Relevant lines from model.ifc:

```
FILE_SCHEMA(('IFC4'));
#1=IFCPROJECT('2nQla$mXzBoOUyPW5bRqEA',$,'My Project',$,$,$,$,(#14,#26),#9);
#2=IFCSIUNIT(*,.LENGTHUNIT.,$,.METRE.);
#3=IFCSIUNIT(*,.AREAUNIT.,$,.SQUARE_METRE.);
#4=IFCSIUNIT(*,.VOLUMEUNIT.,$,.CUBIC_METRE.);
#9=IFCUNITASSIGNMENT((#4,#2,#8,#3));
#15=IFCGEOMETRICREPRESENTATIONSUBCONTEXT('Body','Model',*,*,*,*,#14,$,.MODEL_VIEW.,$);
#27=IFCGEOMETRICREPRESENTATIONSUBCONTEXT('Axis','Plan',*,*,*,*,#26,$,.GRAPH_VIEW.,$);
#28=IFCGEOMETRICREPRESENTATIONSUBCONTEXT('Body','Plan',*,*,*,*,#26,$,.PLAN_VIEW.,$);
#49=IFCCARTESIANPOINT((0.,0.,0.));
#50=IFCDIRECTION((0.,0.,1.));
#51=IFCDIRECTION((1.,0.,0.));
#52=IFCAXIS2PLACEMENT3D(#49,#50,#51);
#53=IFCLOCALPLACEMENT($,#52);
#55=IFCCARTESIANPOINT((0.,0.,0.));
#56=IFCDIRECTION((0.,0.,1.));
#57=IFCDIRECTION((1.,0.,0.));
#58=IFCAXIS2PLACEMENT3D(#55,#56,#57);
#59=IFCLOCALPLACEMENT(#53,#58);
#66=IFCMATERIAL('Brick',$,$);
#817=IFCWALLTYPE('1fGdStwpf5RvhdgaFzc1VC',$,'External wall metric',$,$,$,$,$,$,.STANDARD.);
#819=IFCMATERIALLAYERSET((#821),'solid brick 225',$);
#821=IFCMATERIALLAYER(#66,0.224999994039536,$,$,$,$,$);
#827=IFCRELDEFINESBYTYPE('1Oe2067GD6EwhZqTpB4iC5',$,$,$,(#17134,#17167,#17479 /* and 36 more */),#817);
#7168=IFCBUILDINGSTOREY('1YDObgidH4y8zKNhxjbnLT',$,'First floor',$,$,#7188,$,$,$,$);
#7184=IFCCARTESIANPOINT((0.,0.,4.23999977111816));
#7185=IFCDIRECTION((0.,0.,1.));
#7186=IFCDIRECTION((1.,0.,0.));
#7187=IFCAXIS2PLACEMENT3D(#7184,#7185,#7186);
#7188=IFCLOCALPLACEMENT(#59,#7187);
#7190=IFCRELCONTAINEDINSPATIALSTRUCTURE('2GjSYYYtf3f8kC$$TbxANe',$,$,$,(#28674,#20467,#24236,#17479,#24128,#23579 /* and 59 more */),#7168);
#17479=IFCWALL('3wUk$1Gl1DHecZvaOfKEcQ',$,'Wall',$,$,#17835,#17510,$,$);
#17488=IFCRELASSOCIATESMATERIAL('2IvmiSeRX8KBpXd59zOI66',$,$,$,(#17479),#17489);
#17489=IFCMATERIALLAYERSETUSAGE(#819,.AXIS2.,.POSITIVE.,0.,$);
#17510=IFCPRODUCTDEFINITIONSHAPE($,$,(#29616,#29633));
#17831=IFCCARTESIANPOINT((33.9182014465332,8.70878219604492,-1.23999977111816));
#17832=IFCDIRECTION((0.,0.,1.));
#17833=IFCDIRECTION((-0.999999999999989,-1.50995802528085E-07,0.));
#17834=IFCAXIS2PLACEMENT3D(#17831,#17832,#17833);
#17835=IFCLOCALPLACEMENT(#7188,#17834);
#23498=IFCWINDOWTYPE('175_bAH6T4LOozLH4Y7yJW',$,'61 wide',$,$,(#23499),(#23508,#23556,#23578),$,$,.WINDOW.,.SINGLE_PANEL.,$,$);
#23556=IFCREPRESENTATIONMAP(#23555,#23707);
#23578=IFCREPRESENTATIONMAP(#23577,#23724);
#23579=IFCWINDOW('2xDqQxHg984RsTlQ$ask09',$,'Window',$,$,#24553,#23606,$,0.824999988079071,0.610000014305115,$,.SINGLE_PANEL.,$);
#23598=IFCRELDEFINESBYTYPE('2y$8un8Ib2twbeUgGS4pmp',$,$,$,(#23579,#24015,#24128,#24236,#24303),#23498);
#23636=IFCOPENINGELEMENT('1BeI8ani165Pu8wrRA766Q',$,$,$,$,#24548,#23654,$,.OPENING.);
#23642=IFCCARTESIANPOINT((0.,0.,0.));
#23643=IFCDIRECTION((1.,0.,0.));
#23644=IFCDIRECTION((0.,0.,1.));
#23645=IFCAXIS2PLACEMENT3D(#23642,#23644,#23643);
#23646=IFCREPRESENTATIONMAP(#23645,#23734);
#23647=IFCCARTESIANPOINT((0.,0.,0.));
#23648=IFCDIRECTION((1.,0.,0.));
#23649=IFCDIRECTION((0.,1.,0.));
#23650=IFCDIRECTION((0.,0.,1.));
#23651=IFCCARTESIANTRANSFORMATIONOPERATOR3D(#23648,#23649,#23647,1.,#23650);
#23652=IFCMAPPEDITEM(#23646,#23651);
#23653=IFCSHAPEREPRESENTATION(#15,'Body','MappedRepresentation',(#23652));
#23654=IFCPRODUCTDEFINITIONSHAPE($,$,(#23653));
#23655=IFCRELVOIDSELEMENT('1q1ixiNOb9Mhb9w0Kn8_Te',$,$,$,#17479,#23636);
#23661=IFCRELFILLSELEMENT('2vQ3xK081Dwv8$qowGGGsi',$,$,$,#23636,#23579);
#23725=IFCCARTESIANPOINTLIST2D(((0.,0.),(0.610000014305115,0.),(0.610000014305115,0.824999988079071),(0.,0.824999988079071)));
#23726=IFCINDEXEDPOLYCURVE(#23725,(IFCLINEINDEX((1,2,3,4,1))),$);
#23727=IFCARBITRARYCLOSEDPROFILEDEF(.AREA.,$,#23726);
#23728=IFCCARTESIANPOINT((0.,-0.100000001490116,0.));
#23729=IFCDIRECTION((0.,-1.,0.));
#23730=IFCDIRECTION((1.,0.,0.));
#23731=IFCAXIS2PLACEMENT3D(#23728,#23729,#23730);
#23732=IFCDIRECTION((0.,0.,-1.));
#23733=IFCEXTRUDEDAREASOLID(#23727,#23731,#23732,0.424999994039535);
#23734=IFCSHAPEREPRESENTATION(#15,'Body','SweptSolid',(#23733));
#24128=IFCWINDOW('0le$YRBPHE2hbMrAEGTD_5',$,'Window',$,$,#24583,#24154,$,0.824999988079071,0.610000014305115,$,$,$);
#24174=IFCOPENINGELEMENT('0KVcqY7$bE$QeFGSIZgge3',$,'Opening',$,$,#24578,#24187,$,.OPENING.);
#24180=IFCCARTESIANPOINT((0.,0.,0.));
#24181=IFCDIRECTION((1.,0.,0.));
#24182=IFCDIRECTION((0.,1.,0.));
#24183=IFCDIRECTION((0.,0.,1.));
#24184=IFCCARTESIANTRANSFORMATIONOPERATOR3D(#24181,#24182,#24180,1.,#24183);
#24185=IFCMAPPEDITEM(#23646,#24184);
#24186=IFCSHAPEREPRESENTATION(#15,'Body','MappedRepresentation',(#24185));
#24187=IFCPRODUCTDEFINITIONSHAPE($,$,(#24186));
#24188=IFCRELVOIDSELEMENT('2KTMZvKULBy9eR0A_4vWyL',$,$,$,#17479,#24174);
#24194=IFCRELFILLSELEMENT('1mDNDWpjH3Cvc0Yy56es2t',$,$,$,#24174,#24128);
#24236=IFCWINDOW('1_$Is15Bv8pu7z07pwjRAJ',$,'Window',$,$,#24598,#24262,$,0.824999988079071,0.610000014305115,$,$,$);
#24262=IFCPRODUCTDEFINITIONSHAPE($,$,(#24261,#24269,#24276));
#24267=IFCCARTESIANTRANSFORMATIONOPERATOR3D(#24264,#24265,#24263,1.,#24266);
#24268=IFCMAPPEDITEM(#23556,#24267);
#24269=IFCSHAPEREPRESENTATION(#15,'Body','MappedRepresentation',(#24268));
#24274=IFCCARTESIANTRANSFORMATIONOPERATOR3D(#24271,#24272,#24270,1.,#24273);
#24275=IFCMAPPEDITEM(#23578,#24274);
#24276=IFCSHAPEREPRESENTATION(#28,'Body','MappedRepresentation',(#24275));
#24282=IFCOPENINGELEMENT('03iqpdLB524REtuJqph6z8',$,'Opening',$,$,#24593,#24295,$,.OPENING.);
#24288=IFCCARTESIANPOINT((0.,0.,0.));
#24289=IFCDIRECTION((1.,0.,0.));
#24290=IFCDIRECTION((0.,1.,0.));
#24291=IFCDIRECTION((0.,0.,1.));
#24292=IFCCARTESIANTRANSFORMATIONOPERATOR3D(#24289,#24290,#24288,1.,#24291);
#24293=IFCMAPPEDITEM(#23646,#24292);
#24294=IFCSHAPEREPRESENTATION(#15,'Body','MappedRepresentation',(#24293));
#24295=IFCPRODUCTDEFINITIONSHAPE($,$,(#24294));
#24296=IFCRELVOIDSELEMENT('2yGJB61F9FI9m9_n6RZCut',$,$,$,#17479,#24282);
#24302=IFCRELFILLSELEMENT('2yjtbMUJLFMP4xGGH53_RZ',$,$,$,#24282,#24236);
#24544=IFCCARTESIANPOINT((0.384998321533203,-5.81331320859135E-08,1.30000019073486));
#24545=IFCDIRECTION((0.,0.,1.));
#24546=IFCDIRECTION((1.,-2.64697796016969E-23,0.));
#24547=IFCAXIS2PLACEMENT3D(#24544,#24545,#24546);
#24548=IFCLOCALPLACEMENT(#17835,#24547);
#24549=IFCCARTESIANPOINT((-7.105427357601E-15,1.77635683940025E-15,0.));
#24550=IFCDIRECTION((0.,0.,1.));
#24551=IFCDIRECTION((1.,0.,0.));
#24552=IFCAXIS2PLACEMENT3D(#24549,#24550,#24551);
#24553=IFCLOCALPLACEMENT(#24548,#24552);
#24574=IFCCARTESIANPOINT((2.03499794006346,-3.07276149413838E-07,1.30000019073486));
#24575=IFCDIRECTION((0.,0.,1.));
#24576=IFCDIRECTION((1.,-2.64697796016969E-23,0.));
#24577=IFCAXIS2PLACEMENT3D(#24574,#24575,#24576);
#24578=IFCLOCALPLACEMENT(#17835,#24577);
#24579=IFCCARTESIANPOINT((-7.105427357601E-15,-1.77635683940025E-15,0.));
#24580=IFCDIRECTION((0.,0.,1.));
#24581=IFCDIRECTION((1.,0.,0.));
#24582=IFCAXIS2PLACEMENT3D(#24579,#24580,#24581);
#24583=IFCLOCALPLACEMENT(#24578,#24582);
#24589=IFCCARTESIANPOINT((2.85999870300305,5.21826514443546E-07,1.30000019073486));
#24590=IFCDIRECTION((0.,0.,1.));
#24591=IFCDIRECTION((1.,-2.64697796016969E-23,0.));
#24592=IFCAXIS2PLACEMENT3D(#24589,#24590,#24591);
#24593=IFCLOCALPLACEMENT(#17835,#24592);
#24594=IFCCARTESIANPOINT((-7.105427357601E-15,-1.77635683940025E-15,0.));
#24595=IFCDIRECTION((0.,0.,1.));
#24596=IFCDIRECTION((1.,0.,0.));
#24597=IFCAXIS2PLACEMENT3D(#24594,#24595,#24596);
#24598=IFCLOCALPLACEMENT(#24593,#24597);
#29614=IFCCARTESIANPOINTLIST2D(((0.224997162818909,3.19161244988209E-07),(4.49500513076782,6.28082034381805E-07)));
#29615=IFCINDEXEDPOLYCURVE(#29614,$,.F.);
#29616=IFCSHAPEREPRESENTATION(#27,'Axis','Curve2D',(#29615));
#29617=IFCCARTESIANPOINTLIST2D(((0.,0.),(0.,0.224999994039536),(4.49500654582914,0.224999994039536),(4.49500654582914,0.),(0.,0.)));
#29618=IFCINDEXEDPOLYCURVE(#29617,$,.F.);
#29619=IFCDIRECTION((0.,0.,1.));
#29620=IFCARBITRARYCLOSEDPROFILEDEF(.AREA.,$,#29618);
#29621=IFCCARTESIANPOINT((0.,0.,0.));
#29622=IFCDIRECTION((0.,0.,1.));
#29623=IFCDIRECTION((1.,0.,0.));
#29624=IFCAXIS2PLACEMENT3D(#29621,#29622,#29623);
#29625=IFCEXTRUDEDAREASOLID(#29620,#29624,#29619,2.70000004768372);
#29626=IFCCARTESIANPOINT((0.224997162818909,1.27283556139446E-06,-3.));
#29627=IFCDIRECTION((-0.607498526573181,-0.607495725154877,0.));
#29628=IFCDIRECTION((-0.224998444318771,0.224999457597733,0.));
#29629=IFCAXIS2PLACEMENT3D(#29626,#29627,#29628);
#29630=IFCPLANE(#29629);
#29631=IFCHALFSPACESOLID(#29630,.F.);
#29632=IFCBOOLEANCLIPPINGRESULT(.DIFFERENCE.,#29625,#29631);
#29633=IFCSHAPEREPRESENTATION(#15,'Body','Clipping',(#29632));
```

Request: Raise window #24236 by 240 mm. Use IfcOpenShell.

```python
import numpy as np
import ifcopenshell
import ifcopenshell.api.geometry
import ifcopenshell.util.placement
import ifcopenshell.util.unit

model = ifcopenshell.open("model.ifc")
unit_scale = ifcopenshell.util.unit.calculate_unit_scale(model)

window = model.by_id(24236)
opening = window.FillsVoids[0].RelatingOpeningElement
dz = 0.24 / unit_scale

shift = np.array([0.0, 0.0, dz])
# The window is placed relative to its opening, so it follows when the opening moves.
matrix = ifcopenshell.util.placement.get_local_placement(opening.ObjectPlacement)
matrix[:3, 3] += shift
ifcopenshell.api.geometry.edit_object_placement(
    model, product=opening, matrix=matrix, is_si=False, should_transform_children=True
)

print(f"moved by {dz * unit_scale:+.3f} m")

model.write("model_edited.ifc")
```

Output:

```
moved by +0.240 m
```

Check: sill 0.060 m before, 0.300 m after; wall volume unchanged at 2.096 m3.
